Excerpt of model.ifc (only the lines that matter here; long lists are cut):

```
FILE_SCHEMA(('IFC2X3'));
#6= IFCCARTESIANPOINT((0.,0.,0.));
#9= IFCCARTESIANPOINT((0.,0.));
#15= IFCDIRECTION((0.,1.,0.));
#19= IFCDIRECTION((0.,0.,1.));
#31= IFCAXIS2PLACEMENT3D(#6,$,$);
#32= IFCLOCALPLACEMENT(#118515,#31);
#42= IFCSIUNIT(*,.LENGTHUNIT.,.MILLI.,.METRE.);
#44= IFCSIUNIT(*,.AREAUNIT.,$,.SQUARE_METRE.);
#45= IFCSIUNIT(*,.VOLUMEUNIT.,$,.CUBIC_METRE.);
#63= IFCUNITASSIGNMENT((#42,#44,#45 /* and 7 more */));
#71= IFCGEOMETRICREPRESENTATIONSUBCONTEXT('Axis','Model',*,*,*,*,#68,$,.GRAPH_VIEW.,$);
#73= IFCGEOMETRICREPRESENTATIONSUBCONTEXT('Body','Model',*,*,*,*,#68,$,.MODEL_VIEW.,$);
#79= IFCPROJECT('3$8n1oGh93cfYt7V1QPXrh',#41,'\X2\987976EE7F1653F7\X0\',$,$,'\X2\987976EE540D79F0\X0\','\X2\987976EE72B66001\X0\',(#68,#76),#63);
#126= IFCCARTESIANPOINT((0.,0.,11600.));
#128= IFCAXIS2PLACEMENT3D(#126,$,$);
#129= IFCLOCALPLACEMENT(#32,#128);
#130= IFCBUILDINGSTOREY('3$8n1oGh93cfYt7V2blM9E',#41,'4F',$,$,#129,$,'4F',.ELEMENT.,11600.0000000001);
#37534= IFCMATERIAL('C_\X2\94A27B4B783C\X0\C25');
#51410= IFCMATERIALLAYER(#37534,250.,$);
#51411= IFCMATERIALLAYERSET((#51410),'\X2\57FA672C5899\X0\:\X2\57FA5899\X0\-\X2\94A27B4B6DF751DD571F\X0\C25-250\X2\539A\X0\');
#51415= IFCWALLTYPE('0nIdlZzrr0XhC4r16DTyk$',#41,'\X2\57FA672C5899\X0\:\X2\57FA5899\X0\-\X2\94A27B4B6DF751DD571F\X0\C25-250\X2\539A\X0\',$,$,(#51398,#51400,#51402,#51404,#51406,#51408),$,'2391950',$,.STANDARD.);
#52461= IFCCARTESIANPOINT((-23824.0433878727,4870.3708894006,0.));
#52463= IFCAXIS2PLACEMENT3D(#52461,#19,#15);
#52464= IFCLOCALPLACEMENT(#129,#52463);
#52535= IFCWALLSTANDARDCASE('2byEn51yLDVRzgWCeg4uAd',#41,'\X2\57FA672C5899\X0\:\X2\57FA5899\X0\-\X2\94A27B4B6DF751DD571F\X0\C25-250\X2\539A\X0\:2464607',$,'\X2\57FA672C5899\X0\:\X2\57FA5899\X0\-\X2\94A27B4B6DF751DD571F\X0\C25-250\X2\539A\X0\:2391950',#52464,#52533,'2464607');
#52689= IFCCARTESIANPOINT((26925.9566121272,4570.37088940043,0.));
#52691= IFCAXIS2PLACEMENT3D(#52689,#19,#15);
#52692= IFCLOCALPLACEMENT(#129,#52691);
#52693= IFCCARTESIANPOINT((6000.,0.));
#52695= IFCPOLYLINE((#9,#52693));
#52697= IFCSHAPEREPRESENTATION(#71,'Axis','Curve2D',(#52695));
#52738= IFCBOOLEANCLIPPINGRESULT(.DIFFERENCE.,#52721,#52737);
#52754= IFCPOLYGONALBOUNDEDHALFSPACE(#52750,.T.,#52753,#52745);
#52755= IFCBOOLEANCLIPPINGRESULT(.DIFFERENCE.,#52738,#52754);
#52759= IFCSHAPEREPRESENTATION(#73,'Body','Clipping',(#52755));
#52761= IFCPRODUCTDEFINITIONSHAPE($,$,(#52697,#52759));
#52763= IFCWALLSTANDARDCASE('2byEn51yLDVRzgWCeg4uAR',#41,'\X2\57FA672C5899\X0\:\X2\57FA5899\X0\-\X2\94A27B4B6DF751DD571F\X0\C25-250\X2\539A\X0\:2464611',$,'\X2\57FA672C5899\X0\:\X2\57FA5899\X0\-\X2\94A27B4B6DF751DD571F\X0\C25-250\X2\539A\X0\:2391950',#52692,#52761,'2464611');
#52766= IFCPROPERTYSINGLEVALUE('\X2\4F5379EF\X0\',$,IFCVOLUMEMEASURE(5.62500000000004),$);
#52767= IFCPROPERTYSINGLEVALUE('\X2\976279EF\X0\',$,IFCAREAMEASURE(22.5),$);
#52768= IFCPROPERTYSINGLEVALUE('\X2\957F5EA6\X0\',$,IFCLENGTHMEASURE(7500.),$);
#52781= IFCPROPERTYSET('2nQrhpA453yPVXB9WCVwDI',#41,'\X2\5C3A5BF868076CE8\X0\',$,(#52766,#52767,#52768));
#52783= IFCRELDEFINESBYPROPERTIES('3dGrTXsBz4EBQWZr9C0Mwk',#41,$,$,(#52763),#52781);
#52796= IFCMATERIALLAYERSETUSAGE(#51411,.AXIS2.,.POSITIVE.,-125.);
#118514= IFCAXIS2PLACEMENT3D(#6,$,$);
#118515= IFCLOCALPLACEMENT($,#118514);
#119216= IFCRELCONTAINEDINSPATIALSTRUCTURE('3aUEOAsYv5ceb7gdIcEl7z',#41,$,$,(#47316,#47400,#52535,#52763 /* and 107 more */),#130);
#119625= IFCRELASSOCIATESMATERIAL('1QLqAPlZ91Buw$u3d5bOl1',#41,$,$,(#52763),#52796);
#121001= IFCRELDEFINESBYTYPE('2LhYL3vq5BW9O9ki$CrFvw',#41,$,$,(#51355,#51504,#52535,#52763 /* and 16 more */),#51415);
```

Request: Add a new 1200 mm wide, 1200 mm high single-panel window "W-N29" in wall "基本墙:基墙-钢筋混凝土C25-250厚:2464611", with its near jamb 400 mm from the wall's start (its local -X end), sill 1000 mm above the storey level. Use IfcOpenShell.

```python
import numpy as np
import ifcopenshell
import ifcopenshell.api.feature
import ifcopenshell.api.geometry
import ifcopenshell.api.pset
import ifcopenshell.api.root
import ifcopenshell.api.spatial
import ifcopenshell.api.type
import ifcopenshell.geom
import ifcopenshell.util.element
import ifcopenshell.util.placement
import ifcopenshell.util.representation
import ifcopenshell.util.shape
import ifcopenshell.util.unit

model = ifcopenshell.open("model.ifc")
unit_scale = ifcopenshell.util.unit.calculate_unit_scale(model)
area_scale = ifcopenshell.util.unit.calculate_unit_scale(model, "AREAUNIT")
volume_scale = ifcopenshell.util.unit.calculate_unit_scale(model, "VOLUMEUNIT")
settings = ifcopenshell.geom.settings()


def volume(element):
    """Net volume in cubic metres, openings subtracted."""
    shape = ifcopenshell.geom.create_shape(settings, element)
    return ifcopenshell.util.shape.get_volume(shape.geometry)


wall = model.by_id(52763)
storey = ifcopenshell.util.element.get_container(wall, ifc_class="IfcBuildingStorey")
context = ifcopenshell.util.representation.get_context(model, "Model", "Body", "MODEL_VIEW")
before = volume(wall)

width, height, from_end, sill = 1.2, 1.2, 0.4, 1  # metres

# The wall runs along its own X axis, and the end named is its -X end.
wall_shape = ifcopenshell.geom.create_shape(settings, wall)
x, y, z = ifcopenshell.util.shape.get_vertices(wall_shape.geometry).T
start = x.min() + from_end
face, thickness = float(y.min()), float(y.max() - y.min())
wall_matrix = ifcopenshell.util.placement.get_local_placement(wall.ObjectPlacement)
level = ifcopenshell.util.placement.get_local_placement(storey.ObjectPlacement)[2, 3]


def in_wall(x, y):
    """Placement at x, y metres in the wall's axes, at sill height."""
    matrix = wall_matrix.copy()
    matrix[:, 3] = wall_matrix @ np.array([x / unit_scale, y / unit_scale, 0.0, 1.0])
    matrix[2, 3] = level + sill / unit_scale
    return matrix


# Opening: a box that overshoots both wall faces by 50 mm.
opening = ifcopenshell.api.root.create_entity(model, ifc_class="IfcOpeningElement")
box = ifcopenshell.api.geometry.add_wall_representation(
    model, context=context, length=width, height=height, thickness=thickness + 0.1
)
ifcopenshell.api.geometry.assign_representation(model, product=opening, representation=box)
ifcopenshell.api.geometry.edit_object_placement(model, product=opening, matrix=in_wall(start, face - 0.05), is_si=False)
ifcopenshell.api.feature.add_feature(model, feature=opening, element=wall)

window = ifcopenshell.api.root.create_entity(model, ifc_class="IfcWindow", name="W-N29")
window.OverallWidth, window.OverallHeight = width / unit_scale, height / unit_scale
body = ifcopenshell.api.geometry.add_window_representation(
    model,
    context=context,
    overall_width=window.OverallWidth,
    overall_height=window.OverallHeight,
    partition_type="SINGLE_PANEL",
)
ifcopenshell.api.geometry.assign_representation(model, product=window, representation=body)
ifcopenshell.api.spatial.assign_container(model, products=[window], relating_structure=storey)
fills = ifcopenshell.api.feature.add_filling(model, opening=opening, element=window)
fills.OwnerHistory = window.OwnerHistory  # required in IFC2X3

# IFC2X3 keeps the operation on the window style.
style = ifcopenshell.api.root.create_entity(model, ifc_class="IfcWindowStyle", name="W-N29")
style.OperationType, style.ConstructionType = "SINGLE_PANEL", "NOTDEFINED"
style.ParameterTakesPrecedence = style.Sizeable = False
ifcopenshell.api.type.assign_type(model, related_objects=[window], relating_type=style)

# Centre the window in the wall's thickness.
ifcopenshell.api.geometry.edit_object_placement(model, product=window, matrix=in_wall(start, face), is_si=False)
window_shape = ifcopenshell.geom.create_shape(settings, window)
depth = ifcopenshell.util.shape.get_vertices(window_shape.geometry)[:, 1]
offset = face + thickness / 2 - (depth.min() + depth.max()) / 2
ifcopenshell.api.geometry.edit_object_placement(model, product=window, matrix=in_wall(start, offset), is_si=False)

after = volume(wall)

# Update the wall's stored quantities.
pset = model.by_id(ifcopenshell.util.element.get_pset(wall, "尺寸标注", should_inherit=False)["id"])
ifcopenshell.api.pset.edit_pset(model, pset=pset, properties={
    "体积": model.create_entity("IfcVolumeMeasure", after / volume_scale),
    "面积": model.create_entity("IfcAreaMeasure", after / thickness / area_scale),
})

print(f"wall volume {before:.3f} -> {after:.3f} m3")

model.write("model_edited.ifc")
```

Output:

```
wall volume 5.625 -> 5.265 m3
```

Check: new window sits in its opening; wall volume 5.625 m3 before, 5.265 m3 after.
